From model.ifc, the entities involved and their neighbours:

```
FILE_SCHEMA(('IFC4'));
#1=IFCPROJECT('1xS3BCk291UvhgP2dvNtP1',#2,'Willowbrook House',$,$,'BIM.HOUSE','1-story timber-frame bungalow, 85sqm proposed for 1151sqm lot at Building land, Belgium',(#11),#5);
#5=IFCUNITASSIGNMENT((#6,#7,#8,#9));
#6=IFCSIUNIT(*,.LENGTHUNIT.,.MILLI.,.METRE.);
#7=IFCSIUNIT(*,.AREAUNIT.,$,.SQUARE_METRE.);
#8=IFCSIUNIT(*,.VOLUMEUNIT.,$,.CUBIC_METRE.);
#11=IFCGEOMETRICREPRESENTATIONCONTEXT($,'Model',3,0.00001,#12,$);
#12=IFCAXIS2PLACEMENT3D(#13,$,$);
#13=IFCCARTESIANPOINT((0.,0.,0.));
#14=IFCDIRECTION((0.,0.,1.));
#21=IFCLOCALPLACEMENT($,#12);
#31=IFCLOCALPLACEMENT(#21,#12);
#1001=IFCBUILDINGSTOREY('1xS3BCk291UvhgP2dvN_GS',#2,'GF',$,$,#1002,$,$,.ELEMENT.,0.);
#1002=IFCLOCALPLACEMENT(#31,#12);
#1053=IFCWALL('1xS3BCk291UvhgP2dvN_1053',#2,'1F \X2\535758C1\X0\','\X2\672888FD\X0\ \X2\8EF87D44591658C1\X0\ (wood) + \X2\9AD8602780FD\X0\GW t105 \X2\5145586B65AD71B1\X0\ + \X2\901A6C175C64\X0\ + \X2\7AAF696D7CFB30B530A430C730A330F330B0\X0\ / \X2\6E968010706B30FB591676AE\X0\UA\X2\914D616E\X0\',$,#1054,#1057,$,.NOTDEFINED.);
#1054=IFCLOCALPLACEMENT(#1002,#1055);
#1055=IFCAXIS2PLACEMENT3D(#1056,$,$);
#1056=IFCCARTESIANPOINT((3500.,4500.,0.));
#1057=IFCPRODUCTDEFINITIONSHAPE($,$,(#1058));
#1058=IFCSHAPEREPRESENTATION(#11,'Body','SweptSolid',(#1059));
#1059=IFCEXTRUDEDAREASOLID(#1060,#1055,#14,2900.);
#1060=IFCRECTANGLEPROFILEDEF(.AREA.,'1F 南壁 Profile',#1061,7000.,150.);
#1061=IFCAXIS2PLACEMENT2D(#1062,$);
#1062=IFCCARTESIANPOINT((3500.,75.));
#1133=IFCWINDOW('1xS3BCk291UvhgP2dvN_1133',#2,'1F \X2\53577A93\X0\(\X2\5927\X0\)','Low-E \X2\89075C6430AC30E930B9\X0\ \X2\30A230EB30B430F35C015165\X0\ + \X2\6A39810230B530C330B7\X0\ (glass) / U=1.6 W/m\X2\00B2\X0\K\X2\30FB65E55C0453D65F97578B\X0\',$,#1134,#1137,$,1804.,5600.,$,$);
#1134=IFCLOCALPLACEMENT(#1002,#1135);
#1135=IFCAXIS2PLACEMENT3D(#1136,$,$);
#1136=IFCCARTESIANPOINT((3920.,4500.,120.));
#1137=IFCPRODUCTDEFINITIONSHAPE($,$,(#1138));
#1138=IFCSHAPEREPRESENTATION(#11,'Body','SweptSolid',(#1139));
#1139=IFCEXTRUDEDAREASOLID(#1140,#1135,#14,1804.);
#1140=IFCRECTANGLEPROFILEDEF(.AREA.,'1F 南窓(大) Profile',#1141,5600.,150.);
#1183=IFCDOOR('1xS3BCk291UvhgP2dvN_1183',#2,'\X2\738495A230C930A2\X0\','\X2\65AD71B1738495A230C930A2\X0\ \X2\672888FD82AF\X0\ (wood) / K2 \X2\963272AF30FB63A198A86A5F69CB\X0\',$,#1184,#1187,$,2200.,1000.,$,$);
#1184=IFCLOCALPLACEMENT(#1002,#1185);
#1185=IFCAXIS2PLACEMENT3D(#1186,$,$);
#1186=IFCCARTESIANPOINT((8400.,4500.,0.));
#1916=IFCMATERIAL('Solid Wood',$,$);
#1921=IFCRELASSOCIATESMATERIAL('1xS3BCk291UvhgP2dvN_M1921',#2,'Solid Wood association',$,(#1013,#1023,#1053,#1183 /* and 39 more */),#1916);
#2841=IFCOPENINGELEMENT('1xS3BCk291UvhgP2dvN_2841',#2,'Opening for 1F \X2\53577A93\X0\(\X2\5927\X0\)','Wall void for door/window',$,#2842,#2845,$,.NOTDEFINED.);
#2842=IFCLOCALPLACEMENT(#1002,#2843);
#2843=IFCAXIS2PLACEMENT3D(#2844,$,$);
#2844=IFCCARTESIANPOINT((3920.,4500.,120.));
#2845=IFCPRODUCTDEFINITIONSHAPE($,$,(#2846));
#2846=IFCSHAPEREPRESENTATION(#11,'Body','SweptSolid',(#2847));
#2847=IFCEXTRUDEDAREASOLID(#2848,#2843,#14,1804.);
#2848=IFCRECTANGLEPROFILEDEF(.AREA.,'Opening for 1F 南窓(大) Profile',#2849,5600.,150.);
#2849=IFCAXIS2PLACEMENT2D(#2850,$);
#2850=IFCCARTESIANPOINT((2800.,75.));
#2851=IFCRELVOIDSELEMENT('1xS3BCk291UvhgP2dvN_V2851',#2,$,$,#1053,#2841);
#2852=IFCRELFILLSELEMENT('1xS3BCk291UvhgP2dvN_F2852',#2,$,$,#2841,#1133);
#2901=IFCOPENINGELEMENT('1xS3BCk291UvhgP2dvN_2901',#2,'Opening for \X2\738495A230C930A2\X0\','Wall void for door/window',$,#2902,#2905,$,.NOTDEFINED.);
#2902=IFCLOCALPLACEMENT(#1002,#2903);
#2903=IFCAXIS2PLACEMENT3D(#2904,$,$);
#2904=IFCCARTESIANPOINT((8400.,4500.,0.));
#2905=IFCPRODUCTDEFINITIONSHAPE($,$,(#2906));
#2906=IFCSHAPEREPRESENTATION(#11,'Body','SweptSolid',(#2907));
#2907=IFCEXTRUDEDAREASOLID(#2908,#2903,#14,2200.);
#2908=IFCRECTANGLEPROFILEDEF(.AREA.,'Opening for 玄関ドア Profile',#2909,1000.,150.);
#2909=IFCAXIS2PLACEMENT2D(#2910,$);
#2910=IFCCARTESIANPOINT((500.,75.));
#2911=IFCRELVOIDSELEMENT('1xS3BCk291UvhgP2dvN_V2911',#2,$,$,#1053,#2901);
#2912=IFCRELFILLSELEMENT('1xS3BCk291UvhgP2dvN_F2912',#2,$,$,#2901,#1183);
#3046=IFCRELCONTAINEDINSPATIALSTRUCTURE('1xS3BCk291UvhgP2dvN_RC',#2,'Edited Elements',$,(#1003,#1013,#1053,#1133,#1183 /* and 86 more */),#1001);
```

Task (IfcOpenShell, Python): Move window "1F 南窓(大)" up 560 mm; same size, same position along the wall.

```python
import numpy as np
import ifcopenshell
import ifcopenshell.api.geometry
import ifcopenshell.util.placement
import ifcopenshell.util.unit

model = ifcopenshell.open("model.ifc")
unit_scale = ifcopenshell.util.unit.calculate_unit_scale(model)

window = model.by_guid("1xS3BCk291UvhgP2dvN_1133")
opening = window.FillsVoids[0].RelatingOpeningElement
dz = 560.0

shift = np.array([0.0, 0.0, dz])
# The window is not placed relative to its opening, so move both.
for product in (opening, window):
    matrix = ifcopenshell.util.placement.get_local_placement(product.ObjectPlacement)
    matrix[:3, 3] += shift
    ifcopenshell.api.geometry.edit_object_placement(model, product=product, matrix=matrix, is_si=False)

print(f"moved by {dz * unit_scale:+.3f} m")

model.write("model_rev.ifc")
```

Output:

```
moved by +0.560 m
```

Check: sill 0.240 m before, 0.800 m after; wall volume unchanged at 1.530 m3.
